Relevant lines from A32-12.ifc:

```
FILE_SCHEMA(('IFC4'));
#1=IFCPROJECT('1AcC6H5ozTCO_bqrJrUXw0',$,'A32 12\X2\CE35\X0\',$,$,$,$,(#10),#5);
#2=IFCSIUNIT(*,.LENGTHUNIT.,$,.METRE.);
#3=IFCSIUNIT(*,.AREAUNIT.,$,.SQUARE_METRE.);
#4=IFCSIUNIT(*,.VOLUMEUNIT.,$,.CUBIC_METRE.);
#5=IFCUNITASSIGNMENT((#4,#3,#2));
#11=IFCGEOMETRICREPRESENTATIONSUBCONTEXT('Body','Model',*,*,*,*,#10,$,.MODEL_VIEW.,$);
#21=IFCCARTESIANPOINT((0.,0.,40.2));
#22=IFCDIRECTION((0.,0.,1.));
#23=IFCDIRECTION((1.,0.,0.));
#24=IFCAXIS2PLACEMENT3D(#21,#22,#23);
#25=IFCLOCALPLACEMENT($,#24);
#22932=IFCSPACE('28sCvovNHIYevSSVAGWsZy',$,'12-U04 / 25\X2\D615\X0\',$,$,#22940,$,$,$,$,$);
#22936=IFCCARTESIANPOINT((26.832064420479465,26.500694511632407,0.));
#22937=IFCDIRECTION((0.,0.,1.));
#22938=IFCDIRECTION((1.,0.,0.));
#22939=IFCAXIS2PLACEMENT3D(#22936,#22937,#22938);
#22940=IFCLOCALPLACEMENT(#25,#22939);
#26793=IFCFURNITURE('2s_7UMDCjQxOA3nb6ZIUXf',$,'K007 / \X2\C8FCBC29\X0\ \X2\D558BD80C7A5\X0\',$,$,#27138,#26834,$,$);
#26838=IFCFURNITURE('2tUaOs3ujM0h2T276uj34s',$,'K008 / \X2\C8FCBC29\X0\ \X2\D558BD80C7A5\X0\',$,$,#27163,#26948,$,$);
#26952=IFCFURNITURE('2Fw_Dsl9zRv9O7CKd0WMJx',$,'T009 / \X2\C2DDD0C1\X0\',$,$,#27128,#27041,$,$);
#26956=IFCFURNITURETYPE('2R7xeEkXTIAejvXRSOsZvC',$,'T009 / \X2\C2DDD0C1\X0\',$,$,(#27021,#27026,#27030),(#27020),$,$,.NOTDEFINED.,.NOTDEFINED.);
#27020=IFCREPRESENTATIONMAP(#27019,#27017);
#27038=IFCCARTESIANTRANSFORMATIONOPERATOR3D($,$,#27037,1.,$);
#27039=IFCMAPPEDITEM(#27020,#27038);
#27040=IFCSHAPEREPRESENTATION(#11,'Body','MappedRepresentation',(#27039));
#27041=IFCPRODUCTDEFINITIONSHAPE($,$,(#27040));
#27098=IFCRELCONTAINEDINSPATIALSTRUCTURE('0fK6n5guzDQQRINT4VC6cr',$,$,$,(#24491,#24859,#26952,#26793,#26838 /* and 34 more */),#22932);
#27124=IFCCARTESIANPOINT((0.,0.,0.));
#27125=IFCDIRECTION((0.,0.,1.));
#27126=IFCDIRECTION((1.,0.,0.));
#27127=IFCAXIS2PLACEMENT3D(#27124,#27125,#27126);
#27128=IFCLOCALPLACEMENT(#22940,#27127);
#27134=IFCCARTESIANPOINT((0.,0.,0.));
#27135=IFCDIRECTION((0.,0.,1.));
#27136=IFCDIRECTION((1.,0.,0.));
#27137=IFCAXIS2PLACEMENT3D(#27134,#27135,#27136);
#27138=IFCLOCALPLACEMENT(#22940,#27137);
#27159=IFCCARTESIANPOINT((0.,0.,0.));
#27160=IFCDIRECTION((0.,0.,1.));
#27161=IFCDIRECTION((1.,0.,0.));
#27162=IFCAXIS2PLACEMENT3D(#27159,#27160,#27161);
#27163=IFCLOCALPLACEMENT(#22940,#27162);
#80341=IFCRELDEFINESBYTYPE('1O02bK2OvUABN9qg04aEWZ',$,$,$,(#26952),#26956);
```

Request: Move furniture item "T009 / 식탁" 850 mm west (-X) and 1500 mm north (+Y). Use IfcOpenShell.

```python
import ifcopenshell
import ifcopenshell.api.geometry
import ifcopenshell.util.placement
import ifcopenshell.util.unit

model = ifcopenshell.open("A32-12.ifc")
unit_scale = ifcopenshell.util.unit.calculate_unit_scale(model)

item = model.by_id(26952)
matrix = ifcopenshell.util.placement.get_local_placement(item.ObjectPlacement)
matrix[0, 3] -= 0.85 / unit_scale
matrix[1, 3] += 1.5 / unit_scale
ifcopenshell.api.geometry.edit_object_placement(model, product=item, matrix=matrix, is_si=False)

print(ifcopenshell.util.placement.get_local_placement(item.ObjectPlacement).round(3) + 0.0)

model.write("A32-12_rev.ifc")
```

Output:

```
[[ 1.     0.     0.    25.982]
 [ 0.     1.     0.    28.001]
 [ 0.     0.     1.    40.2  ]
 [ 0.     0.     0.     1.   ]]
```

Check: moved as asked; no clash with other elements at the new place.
